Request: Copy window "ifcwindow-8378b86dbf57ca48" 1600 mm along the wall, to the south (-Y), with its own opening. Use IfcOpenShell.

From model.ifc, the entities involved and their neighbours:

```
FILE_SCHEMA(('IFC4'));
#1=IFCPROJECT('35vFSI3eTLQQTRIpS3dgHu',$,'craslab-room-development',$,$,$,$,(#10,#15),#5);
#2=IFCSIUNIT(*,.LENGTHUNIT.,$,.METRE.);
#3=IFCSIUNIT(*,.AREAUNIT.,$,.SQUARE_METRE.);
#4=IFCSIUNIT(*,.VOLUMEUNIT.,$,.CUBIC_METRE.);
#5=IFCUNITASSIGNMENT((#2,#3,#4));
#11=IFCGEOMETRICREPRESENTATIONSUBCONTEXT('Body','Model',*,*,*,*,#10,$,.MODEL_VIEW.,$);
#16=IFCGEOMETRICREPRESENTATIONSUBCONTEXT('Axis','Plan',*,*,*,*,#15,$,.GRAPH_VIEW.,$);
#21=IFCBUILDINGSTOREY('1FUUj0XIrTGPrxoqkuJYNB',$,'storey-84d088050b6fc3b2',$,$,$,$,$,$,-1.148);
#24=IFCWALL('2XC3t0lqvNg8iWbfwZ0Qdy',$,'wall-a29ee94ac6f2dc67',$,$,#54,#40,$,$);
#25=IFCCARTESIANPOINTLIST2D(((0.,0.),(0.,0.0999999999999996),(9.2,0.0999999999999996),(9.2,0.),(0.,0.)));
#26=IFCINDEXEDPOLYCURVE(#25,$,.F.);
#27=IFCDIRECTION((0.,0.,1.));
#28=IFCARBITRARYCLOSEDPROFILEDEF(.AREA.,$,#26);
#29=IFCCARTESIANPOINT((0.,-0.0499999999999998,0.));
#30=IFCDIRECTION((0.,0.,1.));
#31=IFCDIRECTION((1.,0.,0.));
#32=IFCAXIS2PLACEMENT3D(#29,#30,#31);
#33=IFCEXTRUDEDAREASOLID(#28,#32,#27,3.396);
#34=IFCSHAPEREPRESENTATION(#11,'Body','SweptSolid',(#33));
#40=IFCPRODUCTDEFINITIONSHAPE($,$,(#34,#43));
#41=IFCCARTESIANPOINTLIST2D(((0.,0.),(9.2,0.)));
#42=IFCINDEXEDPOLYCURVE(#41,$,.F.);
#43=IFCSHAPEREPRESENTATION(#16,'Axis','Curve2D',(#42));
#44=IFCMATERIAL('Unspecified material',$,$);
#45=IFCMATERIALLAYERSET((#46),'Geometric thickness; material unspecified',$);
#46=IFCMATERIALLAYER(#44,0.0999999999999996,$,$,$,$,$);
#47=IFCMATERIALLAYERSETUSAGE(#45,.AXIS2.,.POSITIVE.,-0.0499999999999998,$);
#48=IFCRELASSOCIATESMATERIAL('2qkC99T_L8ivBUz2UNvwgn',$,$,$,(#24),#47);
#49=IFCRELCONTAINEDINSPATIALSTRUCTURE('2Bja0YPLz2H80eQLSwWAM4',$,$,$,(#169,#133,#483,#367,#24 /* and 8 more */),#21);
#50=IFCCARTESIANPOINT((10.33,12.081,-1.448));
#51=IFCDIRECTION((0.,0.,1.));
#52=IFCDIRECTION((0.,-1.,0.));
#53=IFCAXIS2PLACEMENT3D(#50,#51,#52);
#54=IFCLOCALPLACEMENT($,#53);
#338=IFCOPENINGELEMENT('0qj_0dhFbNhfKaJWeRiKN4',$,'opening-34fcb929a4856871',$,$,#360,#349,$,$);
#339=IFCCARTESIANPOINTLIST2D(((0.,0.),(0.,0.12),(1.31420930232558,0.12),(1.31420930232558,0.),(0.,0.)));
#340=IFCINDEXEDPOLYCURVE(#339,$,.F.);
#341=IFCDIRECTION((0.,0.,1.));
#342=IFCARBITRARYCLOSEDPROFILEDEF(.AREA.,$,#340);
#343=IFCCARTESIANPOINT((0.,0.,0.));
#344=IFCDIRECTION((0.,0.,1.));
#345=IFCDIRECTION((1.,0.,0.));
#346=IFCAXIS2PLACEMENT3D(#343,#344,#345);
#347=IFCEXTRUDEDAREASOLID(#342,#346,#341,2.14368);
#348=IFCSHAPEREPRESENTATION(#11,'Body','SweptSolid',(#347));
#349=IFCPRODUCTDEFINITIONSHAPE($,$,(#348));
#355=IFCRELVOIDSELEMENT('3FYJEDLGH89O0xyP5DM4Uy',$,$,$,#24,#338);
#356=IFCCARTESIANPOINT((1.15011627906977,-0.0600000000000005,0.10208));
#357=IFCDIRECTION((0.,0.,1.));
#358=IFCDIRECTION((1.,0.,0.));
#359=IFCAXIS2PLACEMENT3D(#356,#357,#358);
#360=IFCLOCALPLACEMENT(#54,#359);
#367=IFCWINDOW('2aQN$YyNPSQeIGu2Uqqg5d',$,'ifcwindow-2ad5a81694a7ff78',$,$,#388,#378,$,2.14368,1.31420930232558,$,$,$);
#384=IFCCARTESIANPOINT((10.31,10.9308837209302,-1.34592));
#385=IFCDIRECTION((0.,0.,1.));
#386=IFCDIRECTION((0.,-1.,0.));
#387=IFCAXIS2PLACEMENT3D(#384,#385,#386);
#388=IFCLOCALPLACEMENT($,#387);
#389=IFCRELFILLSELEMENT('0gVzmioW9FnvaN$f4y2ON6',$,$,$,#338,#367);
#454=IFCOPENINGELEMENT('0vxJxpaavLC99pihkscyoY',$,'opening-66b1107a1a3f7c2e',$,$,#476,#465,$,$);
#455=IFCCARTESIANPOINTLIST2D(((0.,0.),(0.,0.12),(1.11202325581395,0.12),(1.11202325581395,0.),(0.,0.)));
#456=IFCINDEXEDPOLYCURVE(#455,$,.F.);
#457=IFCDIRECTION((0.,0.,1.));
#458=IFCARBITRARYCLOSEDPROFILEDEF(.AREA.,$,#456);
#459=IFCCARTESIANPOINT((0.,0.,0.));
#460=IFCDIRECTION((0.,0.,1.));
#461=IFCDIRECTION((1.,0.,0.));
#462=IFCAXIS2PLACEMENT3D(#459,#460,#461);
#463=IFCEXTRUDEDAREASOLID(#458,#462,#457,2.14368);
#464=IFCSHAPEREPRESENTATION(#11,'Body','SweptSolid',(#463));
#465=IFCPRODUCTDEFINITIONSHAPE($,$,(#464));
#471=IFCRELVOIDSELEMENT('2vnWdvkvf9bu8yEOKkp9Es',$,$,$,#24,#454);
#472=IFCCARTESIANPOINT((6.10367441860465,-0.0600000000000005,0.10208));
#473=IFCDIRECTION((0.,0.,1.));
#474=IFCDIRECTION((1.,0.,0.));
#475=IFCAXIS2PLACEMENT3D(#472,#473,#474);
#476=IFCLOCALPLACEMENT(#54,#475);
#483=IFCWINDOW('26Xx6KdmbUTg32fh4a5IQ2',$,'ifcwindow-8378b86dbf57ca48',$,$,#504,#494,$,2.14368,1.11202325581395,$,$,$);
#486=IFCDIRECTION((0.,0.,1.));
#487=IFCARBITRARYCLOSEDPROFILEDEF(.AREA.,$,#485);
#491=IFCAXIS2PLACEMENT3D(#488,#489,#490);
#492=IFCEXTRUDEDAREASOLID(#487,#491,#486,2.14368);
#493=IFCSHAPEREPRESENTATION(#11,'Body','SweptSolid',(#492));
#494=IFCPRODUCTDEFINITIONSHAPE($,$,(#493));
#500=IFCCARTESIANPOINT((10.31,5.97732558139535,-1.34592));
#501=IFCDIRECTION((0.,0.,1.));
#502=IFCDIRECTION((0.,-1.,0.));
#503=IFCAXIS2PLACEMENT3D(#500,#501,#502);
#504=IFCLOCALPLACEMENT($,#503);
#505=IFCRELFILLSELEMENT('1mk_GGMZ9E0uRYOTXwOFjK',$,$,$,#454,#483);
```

```python
import ifcopenshell
import ifcopenshell.api.feature
import ifcopenshell.api.geometry
import ifcopenshell.api.root
import ifcopenshell.geom
import ifcopenshell.util.element
import ifcopenshell.util.placement
import ifcopenshell.util.shape

model = ifcopenshell.open("model.ifc")
settings = ifcopenshell.geom.settings()


def volume(element):
    """Net volume in cubic metres, openings subtracted."""
    shape = ifcopenshell.geom.create_shape(settings, element)
    return ifcopenshell.util.shape.get_volume(shape.geometry)


window = model.by_id(483)
opening = window.FillsVoids[0].RelatingOpeningElement
wall = opening.VoidsElements[0].RelatingBuildingElement
before = volume(wall)
shift = ifcopenshell.util.placement.get_local_placement(wall.ObjectPlacement)[:3, 0] * 1.6

# copy_class copies the void relationship, type, container and properties, but no geometry.
new_opening = ifcopenshell.api.root.copy_class(model, product=opening)
new_opening.Representation = ifcopenshell.util.element.copy_deep(
    model, opening.Representation, exclude=["IfcGeometricRepresentationContext", "IfcRepresentationMap"]
)
new_window = ifcopenshell.api.root.copy_class(model, product=window)
new_window.Representation = ifcopenshell.util.element.copy_deep(
    model, window.Representation, exclude=["IfcGeometricRepresentationContext", "IfcRepresentationMap"]
)
ifcopenshell.api.feature.add_filling(model, opening=new_opening, element=new_window)

for old, new in ((opening, new_opening), (window, new_window)):
    matrix = ifcopenshell.util.placement.get_local_placement(old.ObjectPlacement)
    matrix[:3, 3] += shift
    ifcopenshell.api.geometry.edit_object_placement(model, product=new, matrix=matrix, is_si=False)

after = volume(wall)

print(f"wall volume {before:.3f} -> {after:.3f} m3")

model.write("model_v2.ifc")
```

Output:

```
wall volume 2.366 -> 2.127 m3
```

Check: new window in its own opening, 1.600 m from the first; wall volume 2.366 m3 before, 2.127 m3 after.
